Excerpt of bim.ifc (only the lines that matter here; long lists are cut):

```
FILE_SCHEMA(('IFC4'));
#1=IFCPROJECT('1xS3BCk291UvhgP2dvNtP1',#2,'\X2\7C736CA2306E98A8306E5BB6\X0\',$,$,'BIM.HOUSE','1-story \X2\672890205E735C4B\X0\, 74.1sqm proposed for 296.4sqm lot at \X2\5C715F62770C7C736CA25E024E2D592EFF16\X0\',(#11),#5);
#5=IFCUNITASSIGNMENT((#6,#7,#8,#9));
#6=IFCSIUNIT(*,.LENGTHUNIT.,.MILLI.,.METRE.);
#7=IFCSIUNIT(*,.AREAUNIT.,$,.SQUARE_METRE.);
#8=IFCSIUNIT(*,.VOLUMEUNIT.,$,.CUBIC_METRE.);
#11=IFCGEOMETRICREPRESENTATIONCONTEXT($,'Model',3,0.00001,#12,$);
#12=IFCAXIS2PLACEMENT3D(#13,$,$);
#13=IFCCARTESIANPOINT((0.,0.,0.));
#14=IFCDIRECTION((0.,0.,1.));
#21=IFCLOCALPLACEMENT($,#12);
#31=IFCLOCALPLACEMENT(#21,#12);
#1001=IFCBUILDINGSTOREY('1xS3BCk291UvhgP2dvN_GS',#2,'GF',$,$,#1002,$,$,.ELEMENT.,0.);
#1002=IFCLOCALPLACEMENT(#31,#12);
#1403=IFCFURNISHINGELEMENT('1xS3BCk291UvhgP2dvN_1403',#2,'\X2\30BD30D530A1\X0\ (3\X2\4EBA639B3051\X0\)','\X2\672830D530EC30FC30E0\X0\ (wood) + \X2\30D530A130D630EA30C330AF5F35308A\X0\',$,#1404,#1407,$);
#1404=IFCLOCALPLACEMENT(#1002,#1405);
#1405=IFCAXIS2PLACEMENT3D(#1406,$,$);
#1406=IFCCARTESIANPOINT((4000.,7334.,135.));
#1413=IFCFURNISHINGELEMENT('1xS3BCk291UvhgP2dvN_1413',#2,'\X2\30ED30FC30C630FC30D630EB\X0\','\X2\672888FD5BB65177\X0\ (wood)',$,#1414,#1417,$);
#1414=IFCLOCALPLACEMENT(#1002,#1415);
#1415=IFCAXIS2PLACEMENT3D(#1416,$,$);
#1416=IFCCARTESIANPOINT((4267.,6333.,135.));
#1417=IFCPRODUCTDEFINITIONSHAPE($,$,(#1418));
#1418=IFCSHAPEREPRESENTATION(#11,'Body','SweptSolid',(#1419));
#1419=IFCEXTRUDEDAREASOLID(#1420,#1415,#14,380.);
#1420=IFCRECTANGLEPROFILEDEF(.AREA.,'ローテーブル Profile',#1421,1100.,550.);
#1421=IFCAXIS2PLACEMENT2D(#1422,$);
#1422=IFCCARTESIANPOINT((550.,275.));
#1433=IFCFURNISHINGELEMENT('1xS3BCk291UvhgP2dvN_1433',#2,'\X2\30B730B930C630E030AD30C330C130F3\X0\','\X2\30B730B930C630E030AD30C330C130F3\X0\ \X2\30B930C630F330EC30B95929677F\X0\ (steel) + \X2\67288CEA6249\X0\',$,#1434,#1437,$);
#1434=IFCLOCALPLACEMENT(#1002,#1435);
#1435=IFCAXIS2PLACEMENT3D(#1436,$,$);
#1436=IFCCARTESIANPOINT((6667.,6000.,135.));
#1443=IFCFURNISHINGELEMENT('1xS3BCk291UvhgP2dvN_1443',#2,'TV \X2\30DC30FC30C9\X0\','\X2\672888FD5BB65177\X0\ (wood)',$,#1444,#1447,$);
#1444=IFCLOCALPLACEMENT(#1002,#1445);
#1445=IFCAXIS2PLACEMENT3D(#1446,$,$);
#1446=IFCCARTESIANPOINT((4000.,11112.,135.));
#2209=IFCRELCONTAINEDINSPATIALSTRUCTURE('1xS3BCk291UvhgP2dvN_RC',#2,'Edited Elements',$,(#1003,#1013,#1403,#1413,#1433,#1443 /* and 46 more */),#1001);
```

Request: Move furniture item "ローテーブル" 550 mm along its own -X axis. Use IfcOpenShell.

```python
import ifcopenshell
import ifcopenshell.api.geometry
import ifcopenshell.util.placement
import ifcopenshell.util.unit

model = ifcopenshell.open("bim.ifc")
unit_scale = ifcopenshell.util.unit.calculate_unit_scale(model)

item = model.by_id(1413)
matrix = ifcopenshell.util.placement.get_local_placement(item.ObjectPlacement)
matrix[:3, 3] -= matrix[:3, 0] * 0.55 / unit_scale
ifcopenshell.api.geometry.edit_object_placement(model, product=item, matrix=matrix, is_si=False)

print(ifcopenshell.util.placement.get_local_placement(item.ObjectPlacement).round(3) + 0.0)

model.write("bim-out.ifc")
```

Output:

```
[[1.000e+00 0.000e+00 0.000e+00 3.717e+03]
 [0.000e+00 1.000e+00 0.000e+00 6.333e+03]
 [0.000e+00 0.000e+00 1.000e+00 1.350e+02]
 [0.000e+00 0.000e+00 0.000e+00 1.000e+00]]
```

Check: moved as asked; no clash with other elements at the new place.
